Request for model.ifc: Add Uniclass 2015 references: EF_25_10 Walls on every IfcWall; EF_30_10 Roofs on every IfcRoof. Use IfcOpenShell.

First a look at what the model holds.

```python
import ifcopenshell

model = ifcopenshell.open("model.ifc")
print(model.schema)
print("classifications:", [c.Name for c in model.by_type("IfcClassification")])
for ifc_class in ("IfcDoor", "IfcRoof", "IfcStair", "IfcWall", "IfcWindow"):
    print(ifc_class, len(model.by_type(ifc_class)))
```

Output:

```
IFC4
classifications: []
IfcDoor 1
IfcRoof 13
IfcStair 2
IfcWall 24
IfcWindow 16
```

```python
import ifcopenshell
import ifcopenshell.api.classification

model = ifcopenshell.open("model.ifc")

system = ifcopenshell.api.classification.add_classification(model, classification="Uniclass 2015")

codes = {
    "IfcWall": ("EF_25_10", "Walls"),
    "IfcRoof": ("EF_30_10", "Roofs"),
}
for ifc_class, (code, name) in codes.items():
    products = model.by_type(ifc_class)
    ifcopenshell.api.classification.add_reference(
        model, products=products, classification=system, identification=code, name=name
    )
    print(code, len(products))

model.write("model_updated.ifc")
```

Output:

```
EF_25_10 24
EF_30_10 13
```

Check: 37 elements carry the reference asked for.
